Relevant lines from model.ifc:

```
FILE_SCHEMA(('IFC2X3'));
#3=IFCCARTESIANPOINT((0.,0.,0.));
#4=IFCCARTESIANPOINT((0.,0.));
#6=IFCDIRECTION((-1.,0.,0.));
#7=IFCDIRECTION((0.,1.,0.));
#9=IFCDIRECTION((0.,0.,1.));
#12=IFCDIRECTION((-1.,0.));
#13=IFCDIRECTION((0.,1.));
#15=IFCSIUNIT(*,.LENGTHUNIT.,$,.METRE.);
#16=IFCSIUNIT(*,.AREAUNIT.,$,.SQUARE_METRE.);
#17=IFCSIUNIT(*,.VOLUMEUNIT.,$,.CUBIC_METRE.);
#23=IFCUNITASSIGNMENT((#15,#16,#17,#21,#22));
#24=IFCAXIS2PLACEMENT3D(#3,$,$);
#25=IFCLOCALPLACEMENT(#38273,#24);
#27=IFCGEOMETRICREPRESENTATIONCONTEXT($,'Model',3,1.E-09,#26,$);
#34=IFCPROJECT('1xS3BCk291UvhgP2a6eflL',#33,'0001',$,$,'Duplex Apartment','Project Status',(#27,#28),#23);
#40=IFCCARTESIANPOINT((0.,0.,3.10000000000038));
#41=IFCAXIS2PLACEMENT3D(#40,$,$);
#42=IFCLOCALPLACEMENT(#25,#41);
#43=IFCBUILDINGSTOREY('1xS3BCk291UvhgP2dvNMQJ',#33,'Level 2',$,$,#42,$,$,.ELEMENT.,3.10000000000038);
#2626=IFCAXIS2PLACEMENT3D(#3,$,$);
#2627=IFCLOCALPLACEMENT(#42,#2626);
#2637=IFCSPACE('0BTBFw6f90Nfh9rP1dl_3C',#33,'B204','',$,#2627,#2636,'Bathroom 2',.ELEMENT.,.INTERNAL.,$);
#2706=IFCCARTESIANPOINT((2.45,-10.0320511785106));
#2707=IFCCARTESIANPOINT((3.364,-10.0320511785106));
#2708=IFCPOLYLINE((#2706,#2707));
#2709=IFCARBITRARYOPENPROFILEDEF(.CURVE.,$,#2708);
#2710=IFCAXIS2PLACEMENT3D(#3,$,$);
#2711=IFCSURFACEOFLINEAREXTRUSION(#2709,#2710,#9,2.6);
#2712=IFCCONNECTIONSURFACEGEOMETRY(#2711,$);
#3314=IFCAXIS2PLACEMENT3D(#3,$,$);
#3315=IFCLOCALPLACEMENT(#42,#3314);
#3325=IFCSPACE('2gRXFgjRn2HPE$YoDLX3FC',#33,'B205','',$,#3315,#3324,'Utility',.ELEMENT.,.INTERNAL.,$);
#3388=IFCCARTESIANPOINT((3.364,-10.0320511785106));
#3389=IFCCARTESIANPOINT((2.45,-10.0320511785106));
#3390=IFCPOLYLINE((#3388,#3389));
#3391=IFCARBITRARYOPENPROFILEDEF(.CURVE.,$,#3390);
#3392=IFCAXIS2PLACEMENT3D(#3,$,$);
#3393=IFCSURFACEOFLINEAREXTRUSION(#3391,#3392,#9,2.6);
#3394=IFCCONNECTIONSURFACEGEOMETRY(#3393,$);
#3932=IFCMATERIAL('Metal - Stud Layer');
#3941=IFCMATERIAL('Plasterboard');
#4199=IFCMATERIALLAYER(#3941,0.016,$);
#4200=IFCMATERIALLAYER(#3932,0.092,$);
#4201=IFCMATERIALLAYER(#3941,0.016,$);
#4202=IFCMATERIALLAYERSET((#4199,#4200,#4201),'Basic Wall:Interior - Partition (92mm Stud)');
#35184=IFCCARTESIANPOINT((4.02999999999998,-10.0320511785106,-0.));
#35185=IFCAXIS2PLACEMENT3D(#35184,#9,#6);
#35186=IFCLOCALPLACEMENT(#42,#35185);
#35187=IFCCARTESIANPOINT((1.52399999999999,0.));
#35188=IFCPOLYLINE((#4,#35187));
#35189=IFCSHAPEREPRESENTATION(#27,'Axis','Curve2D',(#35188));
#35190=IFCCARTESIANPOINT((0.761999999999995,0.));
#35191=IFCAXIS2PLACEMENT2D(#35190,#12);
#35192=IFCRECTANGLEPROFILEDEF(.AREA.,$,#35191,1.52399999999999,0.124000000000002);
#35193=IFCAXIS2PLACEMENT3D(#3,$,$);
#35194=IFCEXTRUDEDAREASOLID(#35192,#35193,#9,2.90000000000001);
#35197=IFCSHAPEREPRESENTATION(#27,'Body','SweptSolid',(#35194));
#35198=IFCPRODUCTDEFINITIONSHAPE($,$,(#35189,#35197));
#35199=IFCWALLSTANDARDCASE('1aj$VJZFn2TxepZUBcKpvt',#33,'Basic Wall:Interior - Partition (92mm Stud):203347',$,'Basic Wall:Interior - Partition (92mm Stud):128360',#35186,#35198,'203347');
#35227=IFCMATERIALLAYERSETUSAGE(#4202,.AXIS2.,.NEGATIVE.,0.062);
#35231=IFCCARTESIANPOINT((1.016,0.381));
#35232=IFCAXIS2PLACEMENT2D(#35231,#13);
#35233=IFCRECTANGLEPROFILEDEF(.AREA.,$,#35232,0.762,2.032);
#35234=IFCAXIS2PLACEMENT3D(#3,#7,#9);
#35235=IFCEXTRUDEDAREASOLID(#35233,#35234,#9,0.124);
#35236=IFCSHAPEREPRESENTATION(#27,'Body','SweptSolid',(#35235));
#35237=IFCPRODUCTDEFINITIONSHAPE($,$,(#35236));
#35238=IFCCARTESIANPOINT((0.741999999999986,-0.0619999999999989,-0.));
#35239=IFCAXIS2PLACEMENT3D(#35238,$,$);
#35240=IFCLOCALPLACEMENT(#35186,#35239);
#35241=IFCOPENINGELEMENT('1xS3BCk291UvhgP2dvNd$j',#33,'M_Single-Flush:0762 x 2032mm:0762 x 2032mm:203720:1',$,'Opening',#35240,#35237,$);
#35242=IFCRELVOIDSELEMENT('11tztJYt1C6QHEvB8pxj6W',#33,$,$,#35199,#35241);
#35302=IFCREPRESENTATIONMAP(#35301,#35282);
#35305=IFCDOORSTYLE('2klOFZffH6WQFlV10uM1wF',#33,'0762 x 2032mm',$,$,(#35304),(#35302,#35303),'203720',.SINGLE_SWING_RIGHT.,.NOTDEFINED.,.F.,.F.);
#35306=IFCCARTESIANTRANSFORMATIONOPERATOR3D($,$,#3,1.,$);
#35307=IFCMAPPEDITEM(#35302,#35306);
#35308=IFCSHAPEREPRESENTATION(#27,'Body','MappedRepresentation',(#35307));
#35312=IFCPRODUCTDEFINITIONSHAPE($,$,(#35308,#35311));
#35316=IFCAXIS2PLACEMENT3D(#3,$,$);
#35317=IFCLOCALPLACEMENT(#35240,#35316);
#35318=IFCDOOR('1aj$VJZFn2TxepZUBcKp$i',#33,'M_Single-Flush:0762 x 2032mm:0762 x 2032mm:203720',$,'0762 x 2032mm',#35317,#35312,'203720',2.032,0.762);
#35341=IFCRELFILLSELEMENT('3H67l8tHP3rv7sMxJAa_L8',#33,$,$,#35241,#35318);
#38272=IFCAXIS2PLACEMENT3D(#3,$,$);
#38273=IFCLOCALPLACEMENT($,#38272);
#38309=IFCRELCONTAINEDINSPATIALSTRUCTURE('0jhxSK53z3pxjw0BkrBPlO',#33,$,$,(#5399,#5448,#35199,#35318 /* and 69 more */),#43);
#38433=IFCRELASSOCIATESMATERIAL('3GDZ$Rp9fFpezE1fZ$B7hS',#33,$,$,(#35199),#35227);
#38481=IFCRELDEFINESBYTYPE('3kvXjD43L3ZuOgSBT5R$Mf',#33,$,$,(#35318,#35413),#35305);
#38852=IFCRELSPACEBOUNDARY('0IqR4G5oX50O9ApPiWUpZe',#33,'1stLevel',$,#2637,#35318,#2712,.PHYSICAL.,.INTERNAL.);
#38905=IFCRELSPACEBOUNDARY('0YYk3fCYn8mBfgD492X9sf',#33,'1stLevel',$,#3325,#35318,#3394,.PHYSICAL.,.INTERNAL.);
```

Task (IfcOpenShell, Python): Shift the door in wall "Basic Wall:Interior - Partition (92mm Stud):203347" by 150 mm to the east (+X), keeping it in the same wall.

```python
import numpy as np
import ifcopenshell
import ifcopenshell.api.geometry
import ifcopenshell.util.placement
import ifcopenshell.util.unit

model = ifcopenshell.open("model.ifc")
unit_scale = ifcopenshell.util.unit.calculate_unit_scale(model)

door = model.by_guid("1aj$VJZFn2TxepZUBcKp$i")
opening = door.FillsVoids[0].RelatingOpeningElement
wall = opening.VoidsElements[0].RelatingBuildingElement

wall_matrix = ifcopenshell.util.placement.get_local_placement(wall.ObjectPlacement)
shift = wall_matrix[:3, 0] * -0.15 / unit_scale
before = ifcopenshell.util.placement.get_local_placement(door.ObjectPlacement)[:3, 3].copy()

# The door is placed relative to its opening, so it follows when the opening moves.
matrix = ifcopenshell.util.placement.get_local_placement(opening.ObjectPlacement)
matrix[:3, 3] += shift
ifcopenshell.api.geometry.edit_object_placement(
    model, product=opening, matrix=matrix, is_si=False, should_transform_children=True
)

# Space boundary surfaces are stored in each space's coordinates; move them too.
for rel in door.ProvidesBoundaries:
    if not rel.ConnectionGeometry:
        continue
    surface = rel.ConnectionGeometry.SurfaceOnRelatingElement
    space_matrix = ifcopenshell.util.placement.get_local_placement(rel.RelatingSpace.ObjectPlacement)
    point = np.array(surface.Position.Location.Coordinates) + space_matrix[:3, :3].T @ shift
    surface.Position = model.createIfcAxis2Placement3D(
        model.createIfcCartesianPoint(point.tolist()), surface.Position.Axis, surface.Position.RefDirection
    )

after = ifcopenshell.util.placement.get_local_placement(door.ObjectPlacement)[:3, 3]
print("door moved by", (after - before).round(3) + 0.0)

model.write("model_rev.ifc")
```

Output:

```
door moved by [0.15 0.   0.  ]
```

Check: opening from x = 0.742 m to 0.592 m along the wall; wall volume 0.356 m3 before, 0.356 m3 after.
